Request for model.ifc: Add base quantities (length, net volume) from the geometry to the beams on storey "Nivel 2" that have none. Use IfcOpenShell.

First a look at what the model holds.

```python
import ifcopenshell
import ifcopenshell.util.element
import ifcopenshell.util.unit

model = ifcopenshell.open("model.ifc")
print(model.schema)
for unit_type in ("LENGTHUNIT", "AREAUNIT", "VOLUMEUNIT"):
    print(unit_type, ifcopenshell.util.unit.calculate_unit_scale(model, unit_type))
storey = next(s for s in model.by_type("IfcBuildingStorey") if s.Name == "Nivel 2")
beams = [e for e in ifcopenshell.util.element.get_decomposition(storey) if e.is_a("IfcBeam")]
for e in sorted(beams, key=lambda e: e.id()):
    print(e.id(), e.is_a(), e.Name, list(ifcopenshell.util.element.get_psets(e, qtos_only=True)), sep=" | ")
```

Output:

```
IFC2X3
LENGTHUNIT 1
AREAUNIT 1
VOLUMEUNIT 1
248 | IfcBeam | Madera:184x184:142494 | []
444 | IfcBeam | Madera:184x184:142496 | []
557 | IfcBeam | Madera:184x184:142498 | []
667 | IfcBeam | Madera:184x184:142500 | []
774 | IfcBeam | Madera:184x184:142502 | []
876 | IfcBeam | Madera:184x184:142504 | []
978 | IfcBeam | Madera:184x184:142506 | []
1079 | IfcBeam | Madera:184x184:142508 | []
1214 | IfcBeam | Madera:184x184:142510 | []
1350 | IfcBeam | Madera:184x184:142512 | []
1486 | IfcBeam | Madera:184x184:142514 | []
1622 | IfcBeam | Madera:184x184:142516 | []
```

```python
import ifcopenshell
import ifcopenshell.api.pset
import ifcopenshell.geom
import ifcopenshell.util.element
import ifcopenshell.util.shape
import ifcopenshell.util.unit

model = ifcopenshell.open("model.ifc")
unit_scale = ifcopenshell.util.unit.calculate_unit_scale(model)
volume_scale = ifcopenshell.util.unit.calculate_unit_scale(model, "VOLUMEUNIT")
settings = ifcopenshell.geom.settings()

storey = next(s for s in model.by_type("IfcBuildingStorey") if s.Name == "Nivel 2")
beams = [e for e in ifcopenshell.util.element.get_decomposition(storey) if e.is_a("IfcBeam")]

for e in sorted(beams, key=lambda e: e.id()):
    if ifcopenshell.util.element.get_psets(e, qtos_only=True, should_inherit=False):
        continue
    # Geometry comes back in metres, in the element's own axes.
    shape = ifcopenshell.geom.create_shape(settings, e)
    values = {
        "Length": ifcopenshell.util.shape.get_max_xyz(shape.geometry) / unit_scale,
        "NetVolume": ifcopenshell.util.shape.get_volume(shape.geometry) / volume_scale,
    }
    qto = ifcopenshell.api.pset.add_qto(model, product=e, name="BaseQuantities")
    ifcopenshell.api.pset.edit_qto(model, qto=qto, properties=values)
    print(e.id(), {k: round(v, 3) for k, v in values.items()})

model.write("model_rev.ifc")
```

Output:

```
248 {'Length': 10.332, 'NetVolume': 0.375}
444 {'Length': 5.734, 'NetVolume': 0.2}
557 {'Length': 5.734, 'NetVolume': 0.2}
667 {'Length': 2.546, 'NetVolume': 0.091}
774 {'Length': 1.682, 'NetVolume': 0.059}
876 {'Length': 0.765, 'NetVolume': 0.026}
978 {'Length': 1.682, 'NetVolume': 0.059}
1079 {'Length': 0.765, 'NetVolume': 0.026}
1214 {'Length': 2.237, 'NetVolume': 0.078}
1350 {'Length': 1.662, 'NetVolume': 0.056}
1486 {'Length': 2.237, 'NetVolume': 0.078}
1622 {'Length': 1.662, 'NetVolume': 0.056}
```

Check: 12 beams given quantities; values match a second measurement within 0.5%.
